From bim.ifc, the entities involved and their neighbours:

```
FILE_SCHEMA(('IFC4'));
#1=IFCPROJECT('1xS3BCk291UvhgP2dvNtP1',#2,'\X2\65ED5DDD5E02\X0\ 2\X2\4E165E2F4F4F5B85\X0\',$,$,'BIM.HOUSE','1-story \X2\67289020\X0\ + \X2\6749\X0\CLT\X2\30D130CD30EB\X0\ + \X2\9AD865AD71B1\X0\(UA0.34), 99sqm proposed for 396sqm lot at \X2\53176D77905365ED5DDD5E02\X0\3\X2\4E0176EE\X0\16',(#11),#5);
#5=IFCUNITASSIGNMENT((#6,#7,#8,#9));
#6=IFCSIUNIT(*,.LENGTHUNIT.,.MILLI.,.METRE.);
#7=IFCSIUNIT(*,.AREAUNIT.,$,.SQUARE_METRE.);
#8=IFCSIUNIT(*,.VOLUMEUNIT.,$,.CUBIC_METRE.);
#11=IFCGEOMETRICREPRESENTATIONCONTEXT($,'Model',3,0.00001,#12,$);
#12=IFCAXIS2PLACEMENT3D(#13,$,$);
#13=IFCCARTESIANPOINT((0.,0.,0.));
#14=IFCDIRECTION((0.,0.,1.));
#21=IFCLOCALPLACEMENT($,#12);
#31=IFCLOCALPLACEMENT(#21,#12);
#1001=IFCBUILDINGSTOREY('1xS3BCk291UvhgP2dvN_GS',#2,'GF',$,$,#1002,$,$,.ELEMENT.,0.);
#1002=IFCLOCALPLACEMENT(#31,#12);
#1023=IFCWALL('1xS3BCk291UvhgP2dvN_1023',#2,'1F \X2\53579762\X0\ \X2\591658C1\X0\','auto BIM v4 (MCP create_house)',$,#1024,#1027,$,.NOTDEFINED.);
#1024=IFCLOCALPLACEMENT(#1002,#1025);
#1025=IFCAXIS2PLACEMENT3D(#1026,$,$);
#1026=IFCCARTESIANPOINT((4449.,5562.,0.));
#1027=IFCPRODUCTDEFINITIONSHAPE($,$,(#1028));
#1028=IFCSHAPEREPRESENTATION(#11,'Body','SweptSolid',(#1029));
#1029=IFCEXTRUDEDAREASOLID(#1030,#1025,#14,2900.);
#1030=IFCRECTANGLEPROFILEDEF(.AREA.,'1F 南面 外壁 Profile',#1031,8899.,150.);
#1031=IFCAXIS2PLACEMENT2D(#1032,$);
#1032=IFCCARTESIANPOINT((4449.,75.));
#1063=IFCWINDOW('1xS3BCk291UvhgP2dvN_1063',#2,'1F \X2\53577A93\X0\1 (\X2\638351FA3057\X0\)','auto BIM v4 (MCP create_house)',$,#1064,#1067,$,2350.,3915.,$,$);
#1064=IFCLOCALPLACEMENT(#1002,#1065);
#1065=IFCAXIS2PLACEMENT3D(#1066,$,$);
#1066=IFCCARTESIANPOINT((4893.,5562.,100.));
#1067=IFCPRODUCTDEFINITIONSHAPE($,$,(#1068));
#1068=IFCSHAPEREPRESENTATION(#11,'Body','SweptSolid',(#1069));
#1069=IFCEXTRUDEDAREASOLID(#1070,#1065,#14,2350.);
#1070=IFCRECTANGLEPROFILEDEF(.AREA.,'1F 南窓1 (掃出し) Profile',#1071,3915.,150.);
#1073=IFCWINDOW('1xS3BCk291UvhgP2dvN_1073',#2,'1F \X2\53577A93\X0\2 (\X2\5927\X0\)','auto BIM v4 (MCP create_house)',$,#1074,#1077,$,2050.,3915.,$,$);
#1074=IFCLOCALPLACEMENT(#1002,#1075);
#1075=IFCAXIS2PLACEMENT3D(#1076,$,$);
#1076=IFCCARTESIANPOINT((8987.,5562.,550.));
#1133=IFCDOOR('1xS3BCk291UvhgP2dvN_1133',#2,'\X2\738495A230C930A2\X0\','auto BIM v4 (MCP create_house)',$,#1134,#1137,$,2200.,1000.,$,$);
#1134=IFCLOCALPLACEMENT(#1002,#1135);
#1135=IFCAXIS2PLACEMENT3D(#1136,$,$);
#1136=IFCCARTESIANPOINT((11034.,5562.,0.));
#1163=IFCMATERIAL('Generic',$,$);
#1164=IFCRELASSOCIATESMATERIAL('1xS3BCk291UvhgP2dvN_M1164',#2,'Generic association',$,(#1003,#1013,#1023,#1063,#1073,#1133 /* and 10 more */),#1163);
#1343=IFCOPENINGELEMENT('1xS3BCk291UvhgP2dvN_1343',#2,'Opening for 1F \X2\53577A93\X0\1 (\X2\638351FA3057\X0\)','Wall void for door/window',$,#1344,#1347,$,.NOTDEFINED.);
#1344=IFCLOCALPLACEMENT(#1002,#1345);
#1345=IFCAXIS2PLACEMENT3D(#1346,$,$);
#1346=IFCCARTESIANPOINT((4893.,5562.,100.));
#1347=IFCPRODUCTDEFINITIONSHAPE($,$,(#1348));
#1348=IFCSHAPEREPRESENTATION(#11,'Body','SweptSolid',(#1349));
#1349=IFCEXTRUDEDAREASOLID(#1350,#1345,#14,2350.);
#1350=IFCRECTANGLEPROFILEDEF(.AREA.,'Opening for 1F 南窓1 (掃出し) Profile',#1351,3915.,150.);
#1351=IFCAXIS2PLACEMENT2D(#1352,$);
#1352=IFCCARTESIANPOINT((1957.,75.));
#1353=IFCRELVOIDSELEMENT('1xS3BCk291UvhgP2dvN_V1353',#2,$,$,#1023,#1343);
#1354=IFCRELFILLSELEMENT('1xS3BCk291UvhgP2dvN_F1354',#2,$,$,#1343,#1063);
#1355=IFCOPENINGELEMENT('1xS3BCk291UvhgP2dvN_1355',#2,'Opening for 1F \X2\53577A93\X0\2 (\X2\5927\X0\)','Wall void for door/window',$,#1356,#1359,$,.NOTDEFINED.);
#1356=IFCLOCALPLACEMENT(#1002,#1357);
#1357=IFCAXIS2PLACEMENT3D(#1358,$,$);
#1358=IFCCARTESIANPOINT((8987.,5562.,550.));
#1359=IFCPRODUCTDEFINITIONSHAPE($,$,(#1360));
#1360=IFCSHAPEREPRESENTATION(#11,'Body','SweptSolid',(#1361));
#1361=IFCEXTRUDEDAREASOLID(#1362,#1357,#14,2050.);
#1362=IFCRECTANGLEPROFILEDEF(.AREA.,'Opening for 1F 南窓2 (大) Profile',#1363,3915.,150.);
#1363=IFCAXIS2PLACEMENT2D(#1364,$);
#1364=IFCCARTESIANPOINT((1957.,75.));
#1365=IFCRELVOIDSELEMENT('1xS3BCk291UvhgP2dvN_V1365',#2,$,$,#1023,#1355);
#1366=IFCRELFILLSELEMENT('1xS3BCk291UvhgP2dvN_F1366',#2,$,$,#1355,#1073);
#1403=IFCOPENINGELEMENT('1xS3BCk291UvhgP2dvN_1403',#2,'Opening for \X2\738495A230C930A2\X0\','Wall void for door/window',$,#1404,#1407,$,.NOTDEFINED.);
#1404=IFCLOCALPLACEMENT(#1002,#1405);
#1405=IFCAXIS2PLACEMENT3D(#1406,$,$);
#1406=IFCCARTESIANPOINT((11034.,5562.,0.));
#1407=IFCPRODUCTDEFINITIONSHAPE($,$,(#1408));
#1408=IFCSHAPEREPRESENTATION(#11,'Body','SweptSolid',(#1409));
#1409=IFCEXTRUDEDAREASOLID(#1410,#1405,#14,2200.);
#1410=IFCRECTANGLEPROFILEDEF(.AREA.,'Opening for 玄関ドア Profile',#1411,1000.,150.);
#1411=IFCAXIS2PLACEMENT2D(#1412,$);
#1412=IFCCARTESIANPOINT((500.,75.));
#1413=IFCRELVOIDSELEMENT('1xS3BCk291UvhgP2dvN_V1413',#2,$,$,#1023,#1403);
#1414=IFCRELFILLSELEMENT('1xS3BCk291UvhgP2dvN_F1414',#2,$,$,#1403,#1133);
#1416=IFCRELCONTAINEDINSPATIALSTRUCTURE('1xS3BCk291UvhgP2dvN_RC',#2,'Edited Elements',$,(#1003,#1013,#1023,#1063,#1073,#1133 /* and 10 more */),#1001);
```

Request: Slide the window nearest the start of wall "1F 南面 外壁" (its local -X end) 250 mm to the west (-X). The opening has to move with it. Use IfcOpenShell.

```python
import ifcopenshell
import ifcopenshell.api.geometry
import ifcopenshell.util.placement
import ifcopenshell.util.unit

model = ifcopenshell.open("bim.ifc")
unit_scale = ifcopenshell.util.unit.calculate_unit_scale(model)

window = model.by_id(1063)
opening = window.FillsVoids[0].RelatingOpeningElement
wall = opening.VoidsElements[0].RelatingBuildingElement

wall_matrix = ifcopenshell.util.placement.get_local_placement(wall.ObjectPlacement)
shift = wall_matrix[:3, 0] * -0.25 / unit_scale
before = ifcopenshell.util.placement.get_local_placement(window.ObjectPlacement)[:3, 3].copy()

# The window is not placed relative to its opening, so move both.
for product in (opening, window):
    matrix = ifcopenshell.util.placement.get_local_placement(product.ObjectPlacement)
    matrix[:3, 3] += shift
    ifcopenshell.api.geometry.edit_object_placement(model, product=product, matrix=matrix, is_si=False)

after = ifcopenshell.util.placement.get_local_placement(window.ObjectPlacement)[:3, 3]
print("window moved by", (after - before).round(3) + 0.0)

model.write("bim_v2.ifc")
```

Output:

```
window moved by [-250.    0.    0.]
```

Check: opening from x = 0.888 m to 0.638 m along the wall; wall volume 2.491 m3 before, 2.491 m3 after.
